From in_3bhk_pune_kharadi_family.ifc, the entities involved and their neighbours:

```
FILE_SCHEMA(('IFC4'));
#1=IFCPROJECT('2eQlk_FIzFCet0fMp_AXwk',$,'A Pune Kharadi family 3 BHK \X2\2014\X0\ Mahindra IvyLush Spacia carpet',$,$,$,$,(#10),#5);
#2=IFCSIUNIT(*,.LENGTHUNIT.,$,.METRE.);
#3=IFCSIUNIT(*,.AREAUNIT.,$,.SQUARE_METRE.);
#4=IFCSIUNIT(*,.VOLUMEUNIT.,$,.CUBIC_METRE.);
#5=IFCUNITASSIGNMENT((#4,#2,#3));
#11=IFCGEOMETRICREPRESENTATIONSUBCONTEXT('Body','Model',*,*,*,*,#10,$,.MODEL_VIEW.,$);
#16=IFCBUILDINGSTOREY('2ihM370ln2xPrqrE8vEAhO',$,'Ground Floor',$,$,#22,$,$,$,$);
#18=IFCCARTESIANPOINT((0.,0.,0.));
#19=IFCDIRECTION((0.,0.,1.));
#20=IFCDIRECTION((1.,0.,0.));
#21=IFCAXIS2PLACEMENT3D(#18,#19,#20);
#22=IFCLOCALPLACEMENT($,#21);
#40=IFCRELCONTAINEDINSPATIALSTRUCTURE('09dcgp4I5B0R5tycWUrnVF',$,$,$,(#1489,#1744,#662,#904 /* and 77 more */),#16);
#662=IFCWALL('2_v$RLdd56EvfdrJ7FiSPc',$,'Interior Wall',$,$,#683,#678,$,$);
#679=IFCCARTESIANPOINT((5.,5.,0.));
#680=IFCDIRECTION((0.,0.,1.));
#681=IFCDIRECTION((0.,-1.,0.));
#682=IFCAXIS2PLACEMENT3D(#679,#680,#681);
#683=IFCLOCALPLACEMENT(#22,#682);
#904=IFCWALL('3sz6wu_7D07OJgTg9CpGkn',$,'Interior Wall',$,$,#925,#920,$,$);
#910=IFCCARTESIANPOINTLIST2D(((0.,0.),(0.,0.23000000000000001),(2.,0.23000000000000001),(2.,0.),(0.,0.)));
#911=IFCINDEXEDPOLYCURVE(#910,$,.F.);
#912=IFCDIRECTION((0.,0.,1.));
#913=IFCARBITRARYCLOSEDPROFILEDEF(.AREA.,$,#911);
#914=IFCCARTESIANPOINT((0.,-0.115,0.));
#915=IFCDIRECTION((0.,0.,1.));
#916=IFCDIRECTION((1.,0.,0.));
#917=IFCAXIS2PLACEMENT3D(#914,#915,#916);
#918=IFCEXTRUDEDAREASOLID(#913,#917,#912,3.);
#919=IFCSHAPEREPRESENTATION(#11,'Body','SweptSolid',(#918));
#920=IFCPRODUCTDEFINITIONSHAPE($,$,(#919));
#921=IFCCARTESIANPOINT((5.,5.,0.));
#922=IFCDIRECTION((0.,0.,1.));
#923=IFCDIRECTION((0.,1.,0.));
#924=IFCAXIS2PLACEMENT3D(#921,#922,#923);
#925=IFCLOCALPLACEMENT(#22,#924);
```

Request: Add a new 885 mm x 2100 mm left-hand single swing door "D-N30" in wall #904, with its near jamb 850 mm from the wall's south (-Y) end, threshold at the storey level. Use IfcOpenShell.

```python
import numpy as np
import ifcopenshell
import ifcopenshell.api.feature
import ifcopenshell.api.geometry
import ifcopenshell.api.root
import ifcopenshell.api.spatial
import ifcopenshell.geom
import ifcopenshell.util.element
import ifcopenshell.util.placement
import ifcopenshell.util.representation
import ifcopenshell.util.shape
import ifcopenshell.util.unit

model = ifcopenshell.open("in_3bhk_pune_kharadi_family.ifc")
unit_scale = ifcopenshell.util.unit.calculate_unit_scale(model)
settings = ifcopenshell.geom.settings()


def volume(element):
    """Net volume in cubic metres, openings subtracted."""
    shape = ifcopenshell.geom.create_shape(settings, element)
    return ifcopenshell.util.shape.get_volume(shape.geometry)


wall = model.by_guid("3sz6wu_7D07OJgTg9CpGkn")
storey = ifcopenshell.util.element.get_container(wall, ifc_class="IfcBuildingStorey")
context = ifcopenshell.util.representation.get_context(model, "Model", "Body", "MODEL_VIEW")
before = volume(wall)

width, height, from_end, sill = 0.885, 2.1, 0.85, 0.0  # metres

# The wall runs along its own X axis, and the end named is its -X end.
wall_shape = ifcopenshell.geom.create_shape(settings, wall)
x, y, z = ifcopenshell.util.shape.get_vertices(wall_shape.geometry).T
start = x.min() + from_end
face, thickness = float(y.min()), float(y.max() - y.min())
wall_matrix = ifcopenshell.util.placement.get_local_placement(wall.ObjectPlacement)
level = ifcopenshell.util.placement.get_local_placement(storey.ObjectPlacement)[2, 3]


def in_wall(x, y):
    """Placement at x, y metres in the wall's axes, at sill height."""
    matrix = wall_matrix.copy()
    matrix[:, 3] = wall_matrix @ np.array([x / unit_scale, y / unit_scale, 0.0, 1.0])
    matrix[2, 3] = level + sill / unit_scale
    return matrix


# Opening: a box that overshoots both wall faces by 50 mm.
opening = ifcopenshell.api.root.create_entity(model, ifc_class="IfcOpeningElement", predefined_type="OPENING")
box = ifcopenshell.api.geometry.add_wall_representation(
    model, context=context, length=width, height=height, thickness=thickness + 0.1
)
ifcopenshell.api.geometry.assign_representation(model, product=opening, representation=box)
ifcopenshell.api.geometry.edit_object_placement(model, product=opening, matrix=in_wall(start, face - 0.05), is_si=False)
ifcopenshell.api.feature.add_feature(model, feature=opening, element=wall)

door = ifcopenshell.api.root.create_entity(model, ifc_class="IfcDoor", name="D-N30", predefined_type="DOOR")
door.OverallWidth, door.OverallHeight = width / unit_scale, height / unit_scale
door.OperationType = "SINGLE_SWING_LEFT"
body = ifcopenshell.api.geometry.add_door_representation(
    model,
    context=context,
    overall_width=door.OverallWidth,
    overall_height=door.OverallHeight,
    operation_type="SINGLE_SWING_LEFT",
    lining_properties={"LiningDepth": thickness / unit_scale, "ThresholdDepth": thickness / unit_scale},
)
ifcopenshell.api.geometry.assign_representation(model, product=door, representation=body)
ifcopenshell.api.spatial.assign_container(model, products=[door], relating_structure=storey)
ifcopenshell.api.feature.add_filling(model, opening=opening, element=door)

# The lining spans the wall, so the door starts at the wall face.
ifcopenshell.api.geometry.edit_object_placement(model, product=door, matrix=in_wall(start, face), is_si=False)

after = volume(wall)

print(f"wall volume {before:.3f} -> {after:.3f} m3")

model.write("in_3bhk_pune_kharadi_family_edited.ifc")
```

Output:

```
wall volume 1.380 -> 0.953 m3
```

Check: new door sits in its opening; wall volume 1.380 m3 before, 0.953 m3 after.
